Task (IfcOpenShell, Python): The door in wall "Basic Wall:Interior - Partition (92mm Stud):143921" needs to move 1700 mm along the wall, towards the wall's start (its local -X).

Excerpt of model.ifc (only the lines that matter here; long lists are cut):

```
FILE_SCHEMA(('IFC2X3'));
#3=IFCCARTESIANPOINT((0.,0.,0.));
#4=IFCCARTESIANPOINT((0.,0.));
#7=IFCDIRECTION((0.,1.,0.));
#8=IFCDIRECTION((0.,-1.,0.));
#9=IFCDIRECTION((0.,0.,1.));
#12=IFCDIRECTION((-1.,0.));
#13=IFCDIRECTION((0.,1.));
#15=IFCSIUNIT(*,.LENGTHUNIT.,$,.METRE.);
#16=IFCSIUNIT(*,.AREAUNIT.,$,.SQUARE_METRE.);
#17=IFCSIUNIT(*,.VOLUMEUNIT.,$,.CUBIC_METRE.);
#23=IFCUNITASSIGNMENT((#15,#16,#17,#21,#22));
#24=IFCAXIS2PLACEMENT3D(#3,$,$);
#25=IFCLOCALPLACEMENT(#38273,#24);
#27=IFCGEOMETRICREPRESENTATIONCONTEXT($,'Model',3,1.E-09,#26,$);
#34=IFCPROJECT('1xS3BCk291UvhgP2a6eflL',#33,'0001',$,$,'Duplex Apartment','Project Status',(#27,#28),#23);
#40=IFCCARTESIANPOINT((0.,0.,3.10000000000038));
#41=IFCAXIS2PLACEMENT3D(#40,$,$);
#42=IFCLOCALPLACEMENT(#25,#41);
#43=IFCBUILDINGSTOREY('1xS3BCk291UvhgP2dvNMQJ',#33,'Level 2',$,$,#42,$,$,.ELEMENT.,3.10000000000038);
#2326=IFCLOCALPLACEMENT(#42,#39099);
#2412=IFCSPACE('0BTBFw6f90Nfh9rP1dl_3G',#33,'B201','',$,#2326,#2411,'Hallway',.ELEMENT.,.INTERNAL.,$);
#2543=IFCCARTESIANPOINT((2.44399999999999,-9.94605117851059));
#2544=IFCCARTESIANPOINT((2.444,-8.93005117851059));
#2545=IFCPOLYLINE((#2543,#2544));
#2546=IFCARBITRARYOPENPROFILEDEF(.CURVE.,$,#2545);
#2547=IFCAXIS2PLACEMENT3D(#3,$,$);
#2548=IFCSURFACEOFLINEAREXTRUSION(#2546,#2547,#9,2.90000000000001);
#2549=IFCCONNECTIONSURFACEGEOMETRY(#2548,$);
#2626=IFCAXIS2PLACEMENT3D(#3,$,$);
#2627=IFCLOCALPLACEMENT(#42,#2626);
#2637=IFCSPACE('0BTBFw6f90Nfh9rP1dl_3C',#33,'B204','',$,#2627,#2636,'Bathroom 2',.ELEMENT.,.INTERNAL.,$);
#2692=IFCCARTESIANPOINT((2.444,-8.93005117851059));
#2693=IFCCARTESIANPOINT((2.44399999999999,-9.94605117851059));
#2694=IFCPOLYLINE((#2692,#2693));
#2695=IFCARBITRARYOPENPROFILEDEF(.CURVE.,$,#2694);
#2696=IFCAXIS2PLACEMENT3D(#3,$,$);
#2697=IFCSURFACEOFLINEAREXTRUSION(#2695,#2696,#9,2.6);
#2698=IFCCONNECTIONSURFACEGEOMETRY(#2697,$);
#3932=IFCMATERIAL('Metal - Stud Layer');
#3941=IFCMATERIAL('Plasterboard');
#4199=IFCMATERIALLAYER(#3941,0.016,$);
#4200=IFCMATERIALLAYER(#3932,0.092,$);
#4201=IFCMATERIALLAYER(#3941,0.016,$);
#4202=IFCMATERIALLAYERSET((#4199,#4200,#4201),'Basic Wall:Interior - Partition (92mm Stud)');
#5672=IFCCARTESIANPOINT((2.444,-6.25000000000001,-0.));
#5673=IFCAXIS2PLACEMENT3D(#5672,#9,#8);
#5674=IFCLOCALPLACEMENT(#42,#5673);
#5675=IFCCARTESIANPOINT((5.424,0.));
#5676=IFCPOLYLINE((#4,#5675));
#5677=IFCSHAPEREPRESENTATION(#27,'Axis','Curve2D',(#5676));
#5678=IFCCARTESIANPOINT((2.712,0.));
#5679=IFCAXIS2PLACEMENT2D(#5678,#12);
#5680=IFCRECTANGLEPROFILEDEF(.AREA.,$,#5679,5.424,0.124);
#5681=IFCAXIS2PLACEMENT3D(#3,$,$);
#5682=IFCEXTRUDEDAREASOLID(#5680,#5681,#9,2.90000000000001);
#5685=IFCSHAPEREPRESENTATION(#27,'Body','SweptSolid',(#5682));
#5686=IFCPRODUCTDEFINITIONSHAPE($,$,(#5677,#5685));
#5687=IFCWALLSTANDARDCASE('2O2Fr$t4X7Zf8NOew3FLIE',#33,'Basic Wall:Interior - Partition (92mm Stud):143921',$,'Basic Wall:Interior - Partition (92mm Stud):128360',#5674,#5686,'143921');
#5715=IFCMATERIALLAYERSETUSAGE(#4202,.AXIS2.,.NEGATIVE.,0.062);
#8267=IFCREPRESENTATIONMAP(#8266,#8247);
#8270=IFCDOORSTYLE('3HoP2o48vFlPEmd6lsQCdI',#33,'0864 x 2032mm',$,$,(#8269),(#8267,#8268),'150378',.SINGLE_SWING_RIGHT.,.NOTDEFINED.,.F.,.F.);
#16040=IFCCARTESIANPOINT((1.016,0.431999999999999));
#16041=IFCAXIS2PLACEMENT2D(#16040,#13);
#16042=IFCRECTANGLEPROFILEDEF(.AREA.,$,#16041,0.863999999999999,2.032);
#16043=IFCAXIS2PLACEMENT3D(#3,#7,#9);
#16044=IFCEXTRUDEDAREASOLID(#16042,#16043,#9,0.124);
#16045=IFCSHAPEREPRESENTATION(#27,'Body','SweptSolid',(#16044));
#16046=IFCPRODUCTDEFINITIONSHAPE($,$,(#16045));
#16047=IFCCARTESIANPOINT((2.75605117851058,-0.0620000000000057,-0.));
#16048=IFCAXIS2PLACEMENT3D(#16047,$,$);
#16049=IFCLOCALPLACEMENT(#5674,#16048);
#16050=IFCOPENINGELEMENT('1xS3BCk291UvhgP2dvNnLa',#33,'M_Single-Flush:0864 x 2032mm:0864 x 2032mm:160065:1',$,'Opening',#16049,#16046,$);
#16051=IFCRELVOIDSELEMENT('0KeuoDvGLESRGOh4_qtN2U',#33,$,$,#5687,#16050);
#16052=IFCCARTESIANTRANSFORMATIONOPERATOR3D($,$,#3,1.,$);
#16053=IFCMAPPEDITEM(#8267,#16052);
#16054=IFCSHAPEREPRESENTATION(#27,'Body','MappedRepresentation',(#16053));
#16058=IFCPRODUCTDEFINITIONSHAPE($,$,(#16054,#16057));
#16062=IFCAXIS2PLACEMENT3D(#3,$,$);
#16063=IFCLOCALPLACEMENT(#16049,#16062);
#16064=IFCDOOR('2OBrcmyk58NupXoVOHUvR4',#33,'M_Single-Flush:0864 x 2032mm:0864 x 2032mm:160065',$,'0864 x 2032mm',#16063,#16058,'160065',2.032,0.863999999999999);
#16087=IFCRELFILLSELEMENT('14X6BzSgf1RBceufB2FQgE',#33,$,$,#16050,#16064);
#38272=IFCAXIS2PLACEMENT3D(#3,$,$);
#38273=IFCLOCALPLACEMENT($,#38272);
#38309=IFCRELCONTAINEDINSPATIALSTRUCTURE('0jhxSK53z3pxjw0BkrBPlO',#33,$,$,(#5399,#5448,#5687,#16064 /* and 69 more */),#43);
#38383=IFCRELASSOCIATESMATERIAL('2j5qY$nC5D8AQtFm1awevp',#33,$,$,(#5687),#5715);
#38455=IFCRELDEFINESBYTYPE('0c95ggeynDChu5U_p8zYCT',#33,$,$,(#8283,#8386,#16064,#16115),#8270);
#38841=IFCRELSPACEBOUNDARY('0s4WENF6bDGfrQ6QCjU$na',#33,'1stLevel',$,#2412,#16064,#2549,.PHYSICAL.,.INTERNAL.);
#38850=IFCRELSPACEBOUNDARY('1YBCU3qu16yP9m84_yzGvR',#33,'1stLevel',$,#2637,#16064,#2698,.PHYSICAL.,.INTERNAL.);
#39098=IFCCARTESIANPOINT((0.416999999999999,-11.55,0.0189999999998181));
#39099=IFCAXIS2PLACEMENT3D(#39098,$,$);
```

```python
import numpy as np
import ifcopenshell
import ifcopenshell.api.geometry
import ifcopenshell.util.placement
import ifcopenshell.util.unit

model = ifcopenshell.open("model.ifc")
unit_scale = ifcopenshell.util.unit.calculate_unit_scale(model)

door = model.by_guid("2OBrcmyk58NupXoVOHUvR4")
opening = door.FillsVoids[0].RelatingOpeningElement
wall = opening.VoidsElements[0].RelatingBuildingElement

wall_matrix = ifcopenshell.util.placement.get_local_placement(wall.ObjectPlacement)
shift = wall_matrix[:3, 0] * -1.7 / unit_scale
before = ifcopenshell.util.placement.get_local_placement(door.ObjectPlacement)[:3, 3].copy()

# The door is placed relative to its opening, so it follows when the opening moves.
matrix = ifcopenshell.util.placement.get_local_placement(opening.ObjectPlacement)
matrix[:3, 3] += shift
ifcopenshell.api.geometry.edit_object_placement(
    model, product=opening, matrix=matrix, is_si=False, should_transform_children=True
)

# Space boundary surfaces are stored in each space's coordinates; move them too.
for rel in door.ProvidesBoundaries:
    if not rel.ConnectionGeometry:
        continue
    surface = rel.ConnectionGeometry.SurfaceOnRelatingElement
    space_matrix = ifcopenshell.util.placement.get_local_placement(rel.RelatingSpace.ObjectPlacement)
    point = np.array(surface.Position.Location.Coordinates) + space_matrix[:3, :3].T @ shift
    surface.Position = model.createIfcAxis2Placement3D(
        model.createIfcCartesianPoint(point.tolist()), surface.Position.Axis, surface.Position.RefDirection
    )

after = ifcopenshell.util.placement.get_local_placement(door.ObjectPlacement)[:3, 3]
print("door moved by", (after - before).round(3) + 0.0)

model.write("model-out.ifc")
```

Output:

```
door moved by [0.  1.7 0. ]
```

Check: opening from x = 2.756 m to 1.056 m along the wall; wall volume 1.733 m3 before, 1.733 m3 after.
